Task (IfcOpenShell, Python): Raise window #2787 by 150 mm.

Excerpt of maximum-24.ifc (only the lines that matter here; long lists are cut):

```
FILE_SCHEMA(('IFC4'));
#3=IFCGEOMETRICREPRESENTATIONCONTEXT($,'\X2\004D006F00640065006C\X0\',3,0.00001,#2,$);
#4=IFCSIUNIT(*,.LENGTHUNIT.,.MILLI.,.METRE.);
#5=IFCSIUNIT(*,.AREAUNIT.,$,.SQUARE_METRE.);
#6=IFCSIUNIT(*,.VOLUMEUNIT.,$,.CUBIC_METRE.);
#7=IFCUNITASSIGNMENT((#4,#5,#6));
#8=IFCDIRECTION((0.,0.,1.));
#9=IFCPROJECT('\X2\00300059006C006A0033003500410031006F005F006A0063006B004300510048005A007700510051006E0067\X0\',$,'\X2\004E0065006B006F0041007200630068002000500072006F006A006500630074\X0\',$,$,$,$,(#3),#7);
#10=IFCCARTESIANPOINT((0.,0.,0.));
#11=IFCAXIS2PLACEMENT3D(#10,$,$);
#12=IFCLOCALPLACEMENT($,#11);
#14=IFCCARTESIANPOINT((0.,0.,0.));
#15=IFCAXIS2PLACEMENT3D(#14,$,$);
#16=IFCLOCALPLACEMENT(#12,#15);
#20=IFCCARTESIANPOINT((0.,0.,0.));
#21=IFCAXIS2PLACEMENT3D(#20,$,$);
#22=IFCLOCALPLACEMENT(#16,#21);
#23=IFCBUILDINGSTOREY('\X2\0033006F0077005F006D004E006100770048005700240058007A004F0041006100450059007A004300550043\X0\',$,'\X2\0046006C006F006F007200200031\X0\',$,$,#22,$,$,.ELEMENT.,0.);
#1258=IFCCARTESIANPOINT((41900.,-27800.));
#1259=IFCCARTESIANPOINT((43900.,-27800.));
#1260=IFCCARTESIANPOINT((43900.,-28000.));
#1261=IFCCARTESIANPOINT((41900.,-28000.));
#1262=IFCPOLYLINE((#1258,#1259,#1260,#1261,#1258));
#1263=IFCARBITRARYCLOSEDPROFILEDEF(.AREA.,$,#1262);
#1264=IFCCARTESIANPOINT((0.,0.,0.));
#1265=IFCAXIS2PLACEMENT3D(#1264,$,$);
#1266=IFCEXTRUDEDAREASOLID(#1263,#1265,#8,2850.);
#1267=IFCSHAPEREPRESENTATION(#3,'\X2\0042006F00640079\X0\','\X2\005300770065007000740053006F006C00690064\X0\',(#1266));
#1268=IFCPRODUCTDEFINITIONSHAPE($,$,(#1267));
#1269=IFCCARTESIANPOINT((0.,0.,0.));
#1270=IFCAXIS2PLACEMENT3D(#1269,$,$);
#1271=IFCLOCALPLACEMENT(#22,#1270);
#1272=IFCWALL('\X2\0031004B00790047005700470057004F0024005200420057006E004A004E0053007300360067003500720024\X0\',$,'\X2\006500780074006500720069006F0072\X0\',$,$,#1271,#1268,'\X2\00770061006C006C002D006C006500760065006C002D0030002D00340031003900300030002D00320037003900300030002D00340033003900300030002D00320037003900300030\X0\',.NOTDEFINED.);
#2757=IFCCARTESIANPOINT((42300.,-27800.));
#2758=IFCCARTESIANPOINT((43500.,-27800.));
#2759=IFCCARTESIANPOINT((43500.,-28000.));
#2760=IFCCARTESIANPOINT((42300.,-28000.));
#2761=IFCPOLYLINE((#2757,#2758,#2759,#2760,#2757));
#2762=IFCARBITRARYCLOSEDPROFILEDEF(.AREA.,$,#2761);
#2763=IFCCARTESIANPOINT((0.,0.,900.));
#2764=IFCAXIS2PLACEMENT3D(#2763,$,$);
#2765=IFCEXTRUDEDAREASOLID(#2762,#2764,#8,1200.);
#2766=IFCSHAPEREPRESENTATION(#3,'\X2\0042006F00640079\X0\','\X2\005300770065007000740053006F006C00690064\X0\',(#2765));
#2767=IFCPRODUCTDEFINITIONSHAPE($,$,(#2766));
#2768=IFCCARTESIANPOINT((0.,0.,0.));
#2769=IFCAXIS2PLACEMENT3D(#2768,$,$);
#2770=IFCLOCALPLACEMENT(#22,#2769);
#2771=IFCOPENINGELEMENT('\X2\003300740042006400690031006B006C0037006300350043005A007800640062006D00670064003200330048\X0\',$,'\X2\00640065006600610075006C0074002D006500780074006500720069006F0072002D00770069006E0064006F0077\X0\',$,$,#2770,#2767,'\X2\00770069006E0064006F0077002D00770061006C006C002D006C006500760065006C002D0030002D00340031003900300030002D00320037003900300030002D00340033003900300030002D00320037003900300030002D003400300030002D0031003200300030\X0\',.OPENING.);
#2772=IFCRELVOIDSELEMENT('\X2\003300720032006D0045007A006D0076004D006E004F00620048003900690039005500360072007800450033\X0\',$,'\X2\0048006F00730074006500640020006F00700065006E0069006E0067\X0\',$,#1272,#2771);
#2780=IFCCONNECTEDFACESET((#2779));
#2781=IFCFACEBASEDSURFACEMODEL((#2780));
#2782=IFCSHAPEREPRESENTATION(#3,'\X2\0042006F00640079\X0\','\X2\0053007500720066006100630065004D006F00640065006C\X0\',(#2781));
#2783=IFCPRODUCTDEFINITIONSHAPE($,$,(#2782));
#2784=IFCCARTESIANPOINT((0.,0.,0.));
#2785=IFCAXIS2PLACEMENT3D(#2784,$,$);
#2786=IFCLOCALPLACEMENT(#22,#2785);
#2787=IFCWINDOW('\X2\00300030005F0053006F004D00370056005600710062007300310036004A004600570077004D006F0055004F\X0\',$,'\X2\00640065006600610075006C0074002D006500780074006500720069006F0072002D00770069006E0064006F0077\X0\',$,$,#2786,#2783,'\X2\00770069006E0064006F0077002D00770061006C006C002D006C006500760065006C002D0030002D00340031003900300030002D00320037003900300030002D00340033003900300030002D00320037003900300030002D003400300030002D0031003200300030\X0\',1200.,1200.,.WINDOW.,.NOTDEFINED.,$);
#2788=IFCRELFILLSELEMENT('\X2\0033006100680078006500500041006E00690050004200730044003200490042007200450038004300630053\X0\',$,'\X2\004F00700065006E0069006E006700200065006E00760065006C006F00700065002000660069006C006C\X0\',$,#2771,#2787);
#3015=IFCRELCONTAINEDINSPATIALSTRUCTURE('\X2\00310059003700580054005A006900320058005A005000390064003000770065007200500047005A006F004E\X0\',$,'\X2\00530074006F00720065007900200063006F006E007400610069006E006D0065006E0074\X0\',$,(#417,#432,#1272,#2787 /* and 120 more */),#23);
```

```python
import numpy as np
import ifcopenshell
import ifcopenshell.api.geometry
import ifcopenshell.util.placement
import ifcopenshell.util.unit

model = ifcopenshell.open("maximum-24.ifc")
unit_scale = ifcopenshell.util.unit.calculate_unit_scale(model)

window = model.by_guid("00_SoM7VVqbs16JFWwMoUO")
opening = window.FillsVoids[0].RelatingOpeningElement
dz = 0.15 / unit_scale

shift = np.array([0.0, 0.0, dz])
# The window is not placed relative to its opening, so move both.
for product in (opening, window):
    matrix = ifcopenshell.util.placement.get_local_placement(product.ObjectPlacement)
    matrix[:3, 3] += shift
    ifcopenshell.api.geometry.edit_object_placement(model, product=product, matrix=matrix, is_si=False)

print(f"moved by {dz * unit_scale:+.3f} m")

model.write("maximum-24_v2.ifc")
```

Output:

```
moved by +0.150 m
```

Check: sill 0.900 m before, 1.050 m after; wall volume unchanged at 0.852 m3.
